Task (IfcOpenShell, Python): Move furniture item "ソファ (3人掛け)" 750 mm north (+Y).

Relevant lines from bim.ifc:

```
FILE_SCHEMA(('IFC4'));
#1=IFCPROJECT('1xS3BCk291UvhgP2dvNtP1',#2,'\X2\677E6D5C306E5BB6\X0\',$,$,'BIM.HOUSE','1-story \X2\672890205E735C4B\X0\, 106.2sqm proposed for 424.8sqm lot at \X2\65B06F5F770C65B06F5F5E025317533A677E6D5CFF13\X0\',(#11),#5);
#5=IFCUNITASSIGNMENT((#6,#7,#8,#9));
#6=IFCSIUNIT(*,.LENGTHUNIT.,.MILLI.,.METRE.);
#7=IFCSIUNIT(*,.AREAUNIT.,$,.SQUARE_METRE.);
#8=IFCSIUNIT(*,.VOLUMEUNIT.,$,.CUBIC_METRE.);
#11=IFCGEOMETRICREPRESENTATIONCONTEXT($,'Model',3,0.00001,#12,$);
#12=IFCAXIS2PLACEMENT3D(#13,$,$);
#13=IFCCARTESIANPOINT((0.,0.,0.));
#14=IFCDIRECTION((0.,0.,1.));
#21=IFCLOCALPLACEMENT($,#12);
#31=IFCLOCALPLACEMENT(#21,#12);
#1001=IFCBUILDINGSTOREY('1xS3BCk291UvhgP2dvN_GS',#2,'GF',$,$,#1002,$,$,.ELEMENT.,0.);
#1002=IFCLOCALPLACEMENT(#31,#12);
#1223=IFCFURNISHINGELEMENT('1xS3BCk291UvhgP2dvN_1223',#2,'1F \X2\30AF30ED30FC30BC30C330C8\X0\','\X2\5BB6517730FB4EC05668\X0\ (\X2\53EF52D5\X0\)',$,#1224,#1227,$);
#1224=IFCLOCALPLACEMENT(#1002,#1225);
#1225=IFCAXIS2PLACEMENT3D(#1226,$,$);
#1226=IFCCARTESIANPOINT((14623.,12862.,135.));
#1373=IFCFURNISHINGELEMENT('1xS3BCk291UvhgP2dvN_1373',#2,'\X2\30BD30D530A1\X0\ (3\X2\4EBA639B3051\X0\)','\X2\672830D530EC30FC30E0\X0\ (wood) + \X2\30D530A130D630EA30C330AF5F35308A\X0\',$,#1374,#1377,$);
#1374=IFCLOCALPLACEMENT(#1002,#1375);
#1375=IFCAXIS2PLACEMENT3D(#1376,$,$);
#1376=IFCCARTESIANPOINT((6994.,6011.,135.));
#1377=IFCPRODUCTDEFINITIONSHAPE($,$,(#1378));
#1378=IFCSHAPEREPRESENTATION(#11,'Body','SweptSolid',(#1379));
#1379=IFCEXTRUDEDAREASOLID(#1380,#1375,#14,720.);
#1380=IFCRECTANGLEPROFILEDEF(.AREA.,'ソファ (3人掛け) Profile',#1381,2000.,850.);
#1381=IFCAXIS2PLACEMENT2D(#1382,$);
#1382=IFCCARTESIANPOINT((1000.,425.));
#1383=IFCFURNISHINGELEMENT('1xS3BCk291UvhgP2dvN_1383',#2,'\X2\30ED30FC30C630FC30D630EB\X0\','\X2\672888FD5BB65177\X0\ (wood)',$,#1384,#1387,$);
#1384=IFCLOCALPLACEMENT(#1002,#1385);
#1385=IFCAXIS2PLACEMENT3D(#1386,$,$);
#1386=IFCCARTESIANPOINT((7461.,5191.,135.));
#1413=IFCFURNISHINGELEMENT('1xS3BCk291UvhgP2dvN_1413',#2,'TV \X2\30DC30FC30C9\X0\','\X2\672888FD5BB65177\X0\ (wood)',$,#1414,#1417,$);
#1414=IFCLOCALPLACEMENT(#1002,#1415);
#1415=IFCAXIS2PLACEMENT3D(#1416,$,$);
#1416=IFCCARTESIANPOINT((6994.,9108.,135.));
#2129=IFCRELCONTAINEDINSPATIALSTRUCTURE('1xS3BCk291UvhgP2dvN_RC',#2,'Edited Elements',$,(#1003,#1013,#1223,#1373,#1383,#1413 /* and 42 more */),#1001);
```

```python
import ifcopenshell
import ifcopenshell.api.geometry
import ifcopenshell.util.placement
import ifcopenshell.util.unit

model = ifcopenshell.open("bim.ifc")
unit_scale = ifcopenshell.util.unit.calculate_unit_scale(model)

item = model.by_guid("1xS3BCk291UvhgP2dvN_1373")
matrix = ifcopenshell.util.placement.get_local_placement(item.ObjectPlacement)
matrix[1, 3] += 0.75 / unit_scale
ifcopenshell.api.geometry.edit_object_placement(model, product=item, matrix=matrix, is_si=False)

print(ifcopenshell.util.placement.get_local_placement(item.ObjectPlacement).round(3) + 0.0)

model.write("bim_updated.ifc")
```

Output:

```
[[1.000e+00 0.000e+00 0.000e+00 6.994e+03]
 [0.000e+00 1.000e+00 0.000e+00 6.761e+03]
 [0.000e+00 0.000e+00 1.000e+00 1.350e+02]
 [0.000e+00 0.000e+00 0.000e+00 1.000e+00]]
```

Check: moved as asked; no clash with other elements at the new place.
